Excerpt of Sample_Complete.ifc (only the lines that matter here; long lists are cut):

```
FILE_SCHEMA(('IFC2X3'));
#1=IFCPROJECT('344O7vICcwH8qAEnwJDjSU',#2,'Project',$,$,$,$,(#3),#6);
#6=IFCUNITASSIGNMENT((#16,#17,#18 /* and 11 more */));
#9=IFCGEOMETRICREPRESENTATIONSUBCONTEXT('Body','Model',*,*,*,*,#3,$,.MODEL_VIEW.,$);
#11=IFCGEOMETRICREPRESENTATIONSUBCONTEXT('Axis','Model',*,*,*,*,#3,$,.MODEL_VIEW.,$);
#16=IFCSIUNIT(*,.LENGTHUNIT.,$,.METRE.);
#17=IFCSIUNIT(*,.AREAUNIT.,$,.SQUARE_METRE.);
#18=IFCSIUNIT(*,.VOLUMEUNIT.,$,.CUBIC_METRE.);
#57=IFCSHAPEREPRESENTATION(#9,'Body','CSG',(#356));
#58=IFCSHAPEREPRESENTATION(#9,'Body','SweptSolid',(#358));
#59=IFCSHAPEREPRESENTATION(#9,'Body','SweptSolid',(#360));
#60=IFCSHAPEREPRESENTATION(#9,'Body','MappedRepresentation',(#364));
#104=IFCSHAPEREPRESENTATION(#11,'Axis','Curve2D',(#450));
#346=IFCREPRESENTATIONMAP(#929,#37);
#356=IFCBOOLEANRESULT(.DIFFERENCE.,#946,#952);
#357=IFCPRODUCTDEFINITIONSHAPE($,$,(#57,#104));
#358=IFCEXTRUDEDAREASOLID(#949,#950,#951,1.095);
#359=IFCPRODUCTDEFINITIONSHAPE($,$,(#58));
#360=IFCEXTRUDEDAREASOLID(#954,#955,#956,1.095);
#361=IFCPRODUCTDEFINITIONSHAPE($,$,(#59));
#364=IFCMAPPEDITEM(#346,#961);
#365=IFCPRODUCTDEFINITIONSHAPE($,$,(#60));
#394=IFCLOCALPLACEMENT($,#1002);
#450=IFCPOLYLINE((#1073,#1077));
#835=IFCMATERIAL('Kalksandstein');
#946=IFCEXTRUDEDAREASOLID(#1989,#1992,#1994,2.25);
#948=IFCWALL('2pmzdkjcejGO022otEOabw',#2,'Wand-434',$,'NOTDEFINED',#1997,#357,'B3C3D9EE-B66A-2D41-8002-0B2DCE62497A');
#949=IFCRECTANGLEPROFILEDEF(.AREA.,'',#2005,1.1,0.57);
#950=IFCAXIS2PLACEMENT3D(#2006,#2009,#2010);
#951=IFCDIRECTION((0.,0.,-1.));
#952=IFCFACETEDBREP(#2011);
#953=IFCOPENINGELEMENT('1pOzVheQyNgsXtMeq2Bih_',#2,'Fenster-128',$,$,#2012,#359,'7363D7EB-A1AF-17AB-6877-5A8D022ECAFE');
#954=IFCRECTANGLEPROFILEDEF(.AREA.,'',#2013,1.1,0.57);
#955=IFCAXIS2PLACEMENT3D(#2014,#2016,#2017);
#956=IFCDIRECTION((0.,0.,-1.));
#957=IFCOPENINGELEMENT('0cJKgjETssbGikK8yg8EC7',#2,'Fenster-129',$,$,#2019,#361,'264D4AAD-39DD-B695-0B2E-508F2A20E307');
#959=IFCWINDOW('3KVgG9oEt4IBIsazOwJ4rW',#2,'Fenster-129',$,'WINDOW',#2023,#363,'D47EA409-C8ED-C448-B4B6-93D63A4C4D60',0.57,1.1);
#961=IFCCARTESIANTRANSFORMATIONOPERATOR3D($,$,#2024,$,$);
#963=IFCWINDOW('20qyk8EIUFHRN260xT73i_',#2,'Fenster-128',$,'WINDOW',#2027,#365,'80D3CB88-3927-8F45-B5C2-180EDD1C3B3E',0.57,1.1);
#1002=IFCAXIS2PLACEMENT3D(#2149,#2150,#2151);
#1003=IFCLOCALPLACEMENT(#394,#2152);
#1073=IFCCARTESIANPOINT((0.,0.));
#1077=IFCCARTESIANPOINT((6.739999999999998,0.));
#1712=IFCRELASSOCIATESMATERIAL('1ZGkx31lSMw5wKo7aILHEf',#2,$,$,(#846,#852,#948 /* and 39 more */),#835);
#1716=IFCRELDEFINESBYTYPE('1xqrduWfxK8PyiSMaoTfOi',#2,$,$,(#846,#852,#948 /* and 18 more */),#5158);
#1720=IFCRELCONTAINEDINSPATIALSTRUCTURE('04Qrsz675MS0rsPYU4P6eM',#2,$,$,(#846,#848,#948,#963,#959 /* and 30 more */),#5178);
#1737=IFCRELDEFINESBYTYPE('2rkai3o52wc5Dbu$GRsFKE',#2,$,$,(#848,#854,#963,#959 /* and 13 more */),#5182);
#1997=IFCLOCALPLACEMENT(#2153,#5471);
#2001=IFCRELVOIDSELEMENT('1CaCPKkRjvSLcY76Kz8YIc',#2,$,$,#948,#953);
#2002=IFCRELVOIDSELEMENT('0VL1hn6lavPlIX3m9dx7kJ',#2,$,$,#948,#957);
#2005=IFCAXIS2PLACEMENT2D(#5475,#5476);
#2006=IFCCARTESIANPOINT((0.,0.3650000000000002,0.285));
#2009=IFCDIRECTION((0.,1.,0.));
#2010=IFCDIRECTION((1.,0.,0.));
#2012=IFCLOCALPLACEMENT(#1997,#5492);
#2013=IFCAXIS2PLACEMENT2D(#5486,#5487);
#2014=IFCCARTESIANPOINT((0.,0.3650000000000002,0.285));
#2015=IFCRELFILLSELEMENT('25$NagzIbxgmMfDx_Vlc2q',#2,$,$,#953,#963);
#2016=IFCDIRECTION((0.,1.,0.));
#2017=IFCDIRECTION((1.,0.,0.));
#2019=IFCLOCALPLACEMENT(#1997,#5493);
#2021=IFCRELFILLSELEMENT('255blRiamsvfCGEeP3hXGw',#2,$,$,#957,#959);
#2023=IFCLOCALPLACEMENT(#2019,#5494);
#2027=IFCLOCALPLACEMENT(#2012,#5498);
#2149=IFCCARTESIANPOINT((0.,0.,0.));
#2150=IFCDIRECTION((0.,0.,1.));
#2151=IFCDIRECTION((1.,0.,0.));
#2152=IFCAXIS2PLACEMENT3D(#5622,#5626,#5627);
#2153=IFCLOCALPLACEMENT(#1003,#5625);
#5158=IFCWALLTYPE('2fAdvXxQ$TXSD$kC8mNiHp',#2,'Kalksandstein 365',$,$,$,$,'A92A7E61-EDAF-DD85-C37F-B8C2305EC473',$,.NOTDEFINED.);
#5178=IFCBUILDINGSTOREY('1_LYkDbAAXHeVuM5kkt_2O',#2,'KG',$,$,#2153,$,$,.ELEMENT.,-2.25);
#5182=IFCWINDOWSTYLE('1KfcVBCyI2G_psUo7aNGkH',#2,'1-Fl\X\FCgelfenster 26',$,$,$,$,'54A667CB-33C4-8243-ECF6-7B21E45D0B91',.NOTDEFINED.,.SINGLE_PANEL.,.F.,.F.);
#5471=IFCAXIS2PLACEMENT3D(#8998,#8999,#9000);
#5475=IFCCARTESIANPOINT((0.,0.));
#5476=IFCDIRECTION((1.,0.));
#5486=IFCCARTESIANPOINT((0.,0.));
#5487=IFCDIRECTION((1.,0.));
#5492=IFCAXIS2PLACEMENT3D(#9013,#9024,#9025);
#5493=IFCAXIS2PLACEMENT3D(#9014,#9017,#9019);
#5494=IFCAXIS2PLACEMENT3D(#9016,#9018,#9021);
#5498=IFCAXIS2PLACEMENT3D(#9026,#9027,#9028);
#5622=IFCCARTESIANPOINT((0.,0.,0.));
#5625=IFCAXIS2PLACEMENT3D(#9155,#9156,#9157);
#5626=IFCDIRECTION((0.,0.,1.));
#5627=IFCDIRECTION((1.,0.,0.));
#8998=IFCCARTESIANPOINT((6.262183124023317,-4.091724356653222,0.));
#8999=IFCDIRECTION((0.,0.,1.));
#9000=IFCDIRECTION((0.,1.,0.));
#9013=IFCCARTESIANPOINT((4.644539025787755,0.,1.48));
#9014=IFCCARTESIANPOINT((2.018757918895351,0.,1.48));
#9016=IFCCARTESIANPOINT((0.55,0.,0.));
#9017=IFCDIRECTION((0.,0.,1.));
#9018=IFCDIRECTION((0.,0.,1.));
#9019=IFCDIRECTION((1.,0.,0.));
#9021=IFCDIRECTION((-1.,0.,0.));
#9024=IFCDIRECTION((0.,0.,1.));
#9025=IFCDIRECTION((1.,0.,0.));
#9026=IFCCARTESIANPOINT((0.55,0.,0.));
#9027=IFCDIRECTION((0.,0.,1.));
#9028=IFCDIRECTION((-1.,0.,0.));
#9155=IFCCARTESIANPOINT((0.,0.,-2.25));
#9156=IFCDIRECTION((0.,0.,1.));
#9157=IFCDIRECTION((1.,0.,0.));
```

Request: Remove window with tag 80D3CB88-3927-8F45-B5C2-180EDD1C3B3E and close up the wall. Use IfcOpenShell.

```python
import ifcopenshell
import ifcopenshell.api.feature
import ifcopenshell.api.root
import ifcopenshell.geom
import ifcopenshell.util.shape

model = ifcopenshell.open("Sample_Complete.ifc")
settings = ifcopenshell.geom.settings()


def volume(element):
    """Net volume in cubic metres, openings subtracted."""
    shape = ifcopenshell.geom.create_shape(settings, element)
    return ifcopenshell.util.shape.get_volume(shape.geometry)


window = model.by_guid("20qyk8EIUFHRN260xT73i_")
opening = window.FillsVoids[0].RelatingOpeningElement
wall = opening.VoidsElements[0].RelatingBuildingElement
before = volume(wall)

ifcopenshell.api.root.remove_product(model, product=window)
ifcopenshell.api.feature.remove_feature(model, feature=opening)

after = volume(wall)

print(f"wall volume {before:.3f} -> {after:.3f} m3")

model.write("Sample_Complete_updated.ifc")
```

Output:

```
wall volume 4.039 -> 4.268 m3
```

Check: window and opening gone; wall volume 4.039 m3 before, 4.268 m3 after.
